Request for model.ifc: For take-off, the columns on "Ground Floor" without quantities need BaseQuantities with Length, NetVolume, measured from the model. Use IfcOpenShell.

First a look at what the model holds.

```python
import ifcopenshell
import ifcopenshell.util.element
import ifcopenshell.util.unit

model = ifcopenshell.open("model.ifc")
print(model.schema)
for unit_type in ("LENGTHUNIT", "AREAUNIT", "VOLUMEUNIT"):
    print(unit_type, ifcopenshell.util.unit.calculate_unit_scale(model, unit_type))
storey = next(s for s in model.by_type("IfcBuildingStorey") if s.Name == "Ground Floor")
columns = [e for e in ifcopenshell.util.element.get_decomposition(storey) if e.is_a("IfcColumn")]
for e in sorted(columns, key=lambda e: e.id()):
    print(e.id(), e.is_a(), e.Name, list(ifcopenshell.util.element.get_psets(e, qtos_only=True)), sep=" | ")
```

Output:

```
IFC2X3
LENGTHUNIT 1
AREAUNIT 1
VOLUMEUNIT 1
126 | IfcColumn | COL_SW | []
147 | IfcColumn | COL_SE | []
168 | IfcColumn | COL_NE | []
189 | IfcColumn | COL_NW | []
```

```python
import ifcopenshell
import ifcopenshell.api.pset
import ifcopenshell.geom
import ifcopenshell.util.element
import ifcopenshell.util.shape
import ifcopenshell.util.unit

model = ifcopenshell.open("model.ifc")
unit_scale = ifcopenshell.util.unit.calculate_unit_scale(model)
volume_scale = ifcopenshell.util.unit.calculate_unit_scale(model, "VOLUMEUNIT")
settings = ifcopenshell.geom.settings()

storey = next(s for s in model.by_type("IfcBuildingStorey") if s.Name == "Ground Floor")
columns = [e for e in ifcopenshell.util.element.get_decomposition(storey) if e.is_a("IfcColumn")]

for e in sorted(columns, key=lambda e: e.id()):
    if ifcopenshell.util.element.get_psets(e, qtos_only=True, should_inherit=False):
        continue
    # Geometry comes back in metres, in the element's own axes.
    shape = ifcopenshell.geom.create_shape(settings, e)
    values = {
        "Length": ifcopenshell.util.shape.get_z(shape.geometry) / unit_scale,
        "NetVolume": ifcopenshell.util.shape.get_volume(shape.geometry) / volume_scale,
    }
    qto = ifcopenshell.api.pset.add_qto(model, product=e, name="BaseQuantities")
    ifcopenshell.api.pset.edit_qto(model, qto=qto, properties=values)
    print(e.id(), {k: round(v, 3) for k, v in values.items()})

model.write("model_rev.ifc")
```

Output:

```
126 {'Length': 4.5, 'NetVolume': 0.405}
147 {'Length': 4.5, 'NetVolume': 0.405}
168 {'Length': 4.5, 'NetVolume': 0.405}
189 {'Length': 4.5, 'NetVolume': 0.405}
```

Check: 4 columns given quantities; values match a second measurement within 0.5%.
